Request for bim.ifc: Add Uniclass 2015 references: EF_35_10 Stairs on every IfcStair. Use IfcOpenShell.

First a look at what the model holds.

```python
import ifcopenshell

model = ifcopenshell.open("bim.ifc")
print(model.schema)
print("classifications:", [c.Name for c in model.by_type("IfcClassification")])
for ifc_class in ("IfcDoor", "IfcRoof", "IfcStair", "IfcWall", "IfcWindow"):
    print(ifc_class, len(model.by_type(ifc_class)))
```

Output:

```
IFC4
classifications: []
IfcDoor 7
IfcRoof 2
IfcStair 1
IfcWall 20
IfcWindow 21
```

```python
import ifcopenshell
import ifcopenshell.api.classification

model = ifcopenshell.open("bim.ifc")

system = ifcopenshell.api.classification.add_classification(model, classification="Uniclass 2015")

codes = {
    "IfcStair": ("EF_35_10", "Stairs"),
}
for ifc_class, (code, name) in codes.items():
    products = model.by_type(ifc_class)
    ifcopenshell.api.classification.add_reference(
        model, products=products, classification=system, identification=code, name=name
    )
    print(code, len(products))

model.write("bim_edited.ifc")
```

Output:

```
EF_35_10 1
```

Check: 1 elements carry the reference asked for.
